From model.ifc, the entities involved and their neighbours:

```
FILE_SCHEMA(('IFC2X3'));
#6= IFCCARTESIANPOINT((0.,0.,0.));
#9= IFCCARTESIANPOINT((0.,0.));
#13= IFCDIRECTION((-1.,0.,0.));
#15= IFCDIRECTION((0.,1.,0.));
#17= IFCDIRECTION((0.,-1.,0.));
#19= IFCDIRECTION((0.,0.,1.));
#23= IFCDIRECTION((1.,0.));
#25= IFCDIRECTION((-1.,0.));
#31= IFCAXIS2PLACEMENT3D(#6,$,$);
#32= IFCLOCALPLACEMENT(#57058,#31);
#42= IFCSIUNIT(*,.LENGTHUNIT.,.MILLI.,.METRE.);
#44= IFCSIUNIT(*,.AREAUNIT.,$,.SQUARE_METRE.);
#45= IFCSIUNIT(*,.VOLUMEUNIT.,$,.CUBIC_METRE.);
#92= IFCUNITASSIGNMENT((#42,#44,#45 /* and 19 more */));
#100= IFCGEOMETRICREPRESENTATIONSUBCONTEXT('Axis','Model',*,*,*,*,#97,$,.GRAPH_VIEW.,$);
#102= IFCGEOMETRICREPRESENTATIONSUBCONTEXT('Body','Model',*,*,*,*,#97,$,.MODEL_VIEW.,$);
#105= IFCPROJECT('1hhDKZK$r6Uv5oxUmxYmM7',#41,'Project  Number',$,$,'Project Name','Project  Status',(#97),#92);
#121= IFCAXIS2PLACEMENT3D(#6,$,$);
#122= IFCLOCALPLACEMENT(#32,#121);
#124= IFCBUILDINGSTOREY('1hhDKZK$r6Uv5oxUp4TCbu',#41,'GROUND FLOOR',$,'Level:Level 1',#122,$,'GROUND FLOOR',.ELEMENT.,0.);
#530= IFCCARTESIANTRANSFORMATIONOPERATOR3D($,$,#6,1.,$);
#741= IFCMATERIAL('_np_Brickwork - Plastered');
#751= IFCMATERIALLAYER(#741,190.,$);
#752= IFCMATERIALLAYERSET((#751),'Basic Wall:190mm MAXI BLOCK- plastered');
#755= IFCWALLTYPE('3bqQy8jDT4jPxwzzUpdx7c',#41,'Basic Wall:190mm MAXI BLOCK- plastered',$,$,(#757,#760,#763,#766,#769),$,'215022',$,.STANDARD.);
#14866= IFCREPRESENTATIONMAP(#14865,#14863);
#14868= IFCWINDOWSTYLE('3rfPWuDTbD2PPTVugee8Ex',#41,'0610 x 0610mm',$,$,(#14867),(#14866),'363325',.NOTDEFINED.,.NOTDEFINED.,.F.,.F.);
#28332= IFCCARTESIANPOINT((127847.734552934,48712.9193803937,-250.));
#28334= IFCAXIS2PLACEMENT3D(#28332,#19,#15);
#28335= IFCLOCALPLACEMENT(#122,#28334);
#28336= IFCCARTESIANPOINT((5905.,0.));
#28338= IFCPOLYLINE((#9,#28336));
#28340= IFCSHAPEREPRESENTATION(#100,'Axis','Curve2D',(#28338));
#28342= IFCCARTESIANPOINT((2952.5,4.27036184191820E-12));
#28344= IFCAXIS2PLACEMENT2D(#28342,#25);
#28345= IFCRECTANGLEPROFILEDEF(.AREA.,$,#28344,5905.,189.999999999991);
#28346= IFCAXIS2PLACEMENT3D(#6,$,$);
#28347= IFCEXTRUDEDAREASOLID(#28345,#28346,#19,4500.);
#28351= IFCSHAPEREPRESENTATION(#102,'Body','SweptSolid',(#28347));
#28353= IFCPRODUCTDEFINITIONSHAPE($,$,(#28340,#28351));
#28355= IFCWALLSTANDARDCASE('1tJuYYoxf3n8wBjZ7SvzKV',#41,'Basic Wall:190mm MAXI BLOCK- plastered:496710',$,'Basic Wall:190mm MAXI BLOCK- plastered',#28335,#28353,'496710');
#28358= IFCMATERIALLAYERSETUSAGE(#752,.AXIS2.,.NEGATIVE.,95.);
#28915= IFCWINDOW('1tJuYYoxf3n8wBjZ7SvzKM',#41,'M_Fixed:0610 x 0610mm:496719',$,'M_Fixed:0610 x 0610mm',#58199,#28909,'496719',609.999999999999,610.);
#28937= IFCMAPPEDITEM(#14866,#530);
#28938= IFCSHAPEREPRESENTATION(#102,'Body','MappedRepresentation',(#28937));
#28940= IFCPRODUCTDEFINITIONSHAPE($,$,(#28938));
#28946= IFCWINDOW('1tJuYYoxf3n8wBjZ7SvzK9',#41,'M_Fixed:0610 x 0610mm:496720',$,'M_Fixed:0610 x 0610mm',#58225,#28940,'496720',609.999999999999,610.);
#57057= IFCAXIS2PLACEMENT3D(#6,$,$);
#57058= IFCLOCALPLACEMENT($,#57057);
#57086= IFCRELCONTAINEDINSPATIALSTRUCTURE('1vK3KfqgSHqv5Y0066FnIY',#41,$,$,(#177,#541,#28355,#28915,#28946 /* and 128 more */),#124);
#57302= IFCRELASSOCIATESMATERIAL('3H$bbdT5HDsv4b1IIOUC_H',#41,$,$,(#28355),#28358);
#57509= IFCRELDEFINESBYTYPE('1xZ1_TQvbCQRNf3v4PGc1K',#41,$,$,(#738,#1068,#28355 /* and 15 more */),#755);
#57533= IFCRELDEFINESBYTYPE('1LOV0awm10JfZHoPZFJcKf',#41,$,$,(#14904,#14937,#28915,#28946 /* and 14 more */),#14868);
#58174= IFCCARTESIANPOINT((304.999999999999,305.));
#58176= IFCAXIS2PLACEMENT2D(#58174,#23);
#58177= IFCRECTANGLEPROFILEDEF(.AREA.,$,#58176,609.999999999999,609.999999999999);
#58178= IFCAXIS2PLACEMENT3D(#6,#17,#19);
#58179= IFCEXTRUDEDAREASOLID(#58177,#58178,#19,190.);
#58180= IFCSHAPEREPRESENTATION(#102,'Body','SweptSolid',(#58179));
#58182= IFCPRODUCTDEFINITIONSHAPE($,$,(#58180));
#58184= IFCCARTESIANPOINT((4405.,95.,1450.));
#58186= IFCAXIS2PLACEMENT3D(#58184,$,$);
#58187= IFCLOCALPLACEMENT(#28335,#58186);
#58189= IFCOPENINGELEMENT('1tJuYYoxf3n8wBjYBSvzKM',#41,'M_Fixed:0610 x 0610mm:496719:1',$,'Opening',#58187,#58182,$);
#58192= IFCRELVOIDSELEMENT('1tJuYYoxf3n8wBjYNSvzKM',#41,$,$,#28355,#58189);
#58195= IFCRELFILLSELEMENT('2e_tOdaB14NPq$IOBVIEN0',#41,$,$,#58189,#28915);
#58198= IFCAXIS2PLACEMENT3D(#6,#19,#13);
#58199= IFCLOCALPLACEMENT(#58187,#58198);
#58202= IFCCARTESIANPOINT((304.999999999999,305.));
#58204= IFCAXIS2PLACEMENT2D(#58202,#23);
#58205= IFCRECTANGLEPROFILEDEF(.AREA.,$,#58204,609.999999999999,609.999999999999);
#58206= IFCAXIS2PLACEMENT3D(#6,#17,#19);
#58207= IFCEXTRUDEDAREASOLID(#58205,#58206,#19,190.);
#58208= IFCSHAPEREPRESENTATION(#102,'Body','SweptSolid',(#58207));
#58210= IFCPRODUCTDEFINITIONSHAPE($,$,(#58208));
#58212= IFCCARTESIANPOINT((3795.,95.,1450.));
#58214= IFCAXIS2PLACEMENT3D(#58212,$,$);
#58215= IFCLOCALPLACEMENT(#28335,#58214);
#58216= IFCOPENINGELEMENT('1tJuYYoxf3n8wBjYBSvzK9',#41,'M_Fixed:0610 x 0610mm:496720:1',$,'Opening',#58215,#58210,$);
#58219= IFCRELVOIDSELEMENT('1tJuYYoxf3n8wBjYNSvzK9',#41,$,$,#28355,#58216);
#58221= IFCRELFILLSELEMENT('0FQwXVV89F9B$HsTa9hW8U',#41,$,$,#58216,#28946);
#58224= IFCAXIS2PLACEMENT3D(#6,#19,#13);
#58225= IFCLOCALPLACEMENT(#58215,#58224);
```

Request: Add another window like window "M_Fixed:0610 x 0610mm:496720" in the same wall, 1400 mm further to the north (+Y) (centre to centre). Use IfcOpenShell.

```python
import ifcopenshell
import ifcopenshell.api.feature
import ifcopenshell.api.geometry
import ifcopenshell.api.root
import ifcopenshell.geom
import ifcopenshell.util.element
import ifcopenshell.util.placement
import ifcopenshell.util.shape

model = ifcopenshell.open("model.ifc")
settings = ifcopenshell.geom.settings()


def volume(element):
    """Net volume in cubic metres, openings subtracted."""
    shape = ifcopenshell.geom.create_shape(settings, element)
    return ifcopenshell.util.shape.get_volume(shape.geometry)


def reuse_history(source, copy):
    """copy_class also copies each property set's owner history, people and application; keep the originals."""
    for rel in copy.IsDefinedBy:
        if rel.is_a("IfcRelDefinesByProperties") and (history := rel.RelatingPropertyDefinition.OwnerHistory):
            rel.RelatingPropertyDefinition.OwnerHistory = source.OwnerHistory
            ifcopenshell.util.element.remove_deep2(model, history)


window = model.by_guid("1tJuYYoxf3n8wBjZ7SvzK9")
opening = window.FillsVoids[0].RelatingOpeningElement
wall = opening.VoidsElements[0].RelatingBuildingElement
before = volume(wall)
shift = ifcopenshell.util.placement.get_local_placement(wall.ObjectPlacement)[:3, 0] * 1400.0

# copy_class copies the void relationship, type, container and properties, but no geometry.
new_opening = ifcopenshell.api.root.copy_class(model, product=opening)
new_opening.Representation = ifcopenshell.util.element.copy_deep(
    model, opening.Representation, exclude=["IfcGeometricRepresentationContext", "IfcRepresentationMap"]
)
new_opening.Name = "M_Fixed:0610 x 0610mm"
new_window = ifcopenshell.api.root.copy_class(model, product=window)
new_window.Representation = ifcopenshell.util.element.copy_deep(
    model, window.Representation, exclude=["IfcGeometricRepresentationContext", "IfcRepresentationMap"]
)
new_window.Name = "M_Fixed:0610 x 0610mm"
new_window.Tag = None
reuse_history(window, new_window)
fills = ifcopenshell.api.feature.add_filling(model, opening=new_opening, element=new_window)
fills.OwnerHistory = new_window.OwnerHistory  # required in IFC2X3

for old, new in ((opening, new_opening), (window, new_window)):
    matrix = ifcopenshell.util.placement.get_local_placement(old.ObjectPlacement)
    matrix[:3, 3] += shift
    ifcopenshell.api.geometry.edit_object_placement(model, product=new, matrix=matrix, is_si=False)

after = volume(wall)

print(f"wall volume {before:.3f} -> {after:.3f} m3")

model.write("model_v2.ifc")
```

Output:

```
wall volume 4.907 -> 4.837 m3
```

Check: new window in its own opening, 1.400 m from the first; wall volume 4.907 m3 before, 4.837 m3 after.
